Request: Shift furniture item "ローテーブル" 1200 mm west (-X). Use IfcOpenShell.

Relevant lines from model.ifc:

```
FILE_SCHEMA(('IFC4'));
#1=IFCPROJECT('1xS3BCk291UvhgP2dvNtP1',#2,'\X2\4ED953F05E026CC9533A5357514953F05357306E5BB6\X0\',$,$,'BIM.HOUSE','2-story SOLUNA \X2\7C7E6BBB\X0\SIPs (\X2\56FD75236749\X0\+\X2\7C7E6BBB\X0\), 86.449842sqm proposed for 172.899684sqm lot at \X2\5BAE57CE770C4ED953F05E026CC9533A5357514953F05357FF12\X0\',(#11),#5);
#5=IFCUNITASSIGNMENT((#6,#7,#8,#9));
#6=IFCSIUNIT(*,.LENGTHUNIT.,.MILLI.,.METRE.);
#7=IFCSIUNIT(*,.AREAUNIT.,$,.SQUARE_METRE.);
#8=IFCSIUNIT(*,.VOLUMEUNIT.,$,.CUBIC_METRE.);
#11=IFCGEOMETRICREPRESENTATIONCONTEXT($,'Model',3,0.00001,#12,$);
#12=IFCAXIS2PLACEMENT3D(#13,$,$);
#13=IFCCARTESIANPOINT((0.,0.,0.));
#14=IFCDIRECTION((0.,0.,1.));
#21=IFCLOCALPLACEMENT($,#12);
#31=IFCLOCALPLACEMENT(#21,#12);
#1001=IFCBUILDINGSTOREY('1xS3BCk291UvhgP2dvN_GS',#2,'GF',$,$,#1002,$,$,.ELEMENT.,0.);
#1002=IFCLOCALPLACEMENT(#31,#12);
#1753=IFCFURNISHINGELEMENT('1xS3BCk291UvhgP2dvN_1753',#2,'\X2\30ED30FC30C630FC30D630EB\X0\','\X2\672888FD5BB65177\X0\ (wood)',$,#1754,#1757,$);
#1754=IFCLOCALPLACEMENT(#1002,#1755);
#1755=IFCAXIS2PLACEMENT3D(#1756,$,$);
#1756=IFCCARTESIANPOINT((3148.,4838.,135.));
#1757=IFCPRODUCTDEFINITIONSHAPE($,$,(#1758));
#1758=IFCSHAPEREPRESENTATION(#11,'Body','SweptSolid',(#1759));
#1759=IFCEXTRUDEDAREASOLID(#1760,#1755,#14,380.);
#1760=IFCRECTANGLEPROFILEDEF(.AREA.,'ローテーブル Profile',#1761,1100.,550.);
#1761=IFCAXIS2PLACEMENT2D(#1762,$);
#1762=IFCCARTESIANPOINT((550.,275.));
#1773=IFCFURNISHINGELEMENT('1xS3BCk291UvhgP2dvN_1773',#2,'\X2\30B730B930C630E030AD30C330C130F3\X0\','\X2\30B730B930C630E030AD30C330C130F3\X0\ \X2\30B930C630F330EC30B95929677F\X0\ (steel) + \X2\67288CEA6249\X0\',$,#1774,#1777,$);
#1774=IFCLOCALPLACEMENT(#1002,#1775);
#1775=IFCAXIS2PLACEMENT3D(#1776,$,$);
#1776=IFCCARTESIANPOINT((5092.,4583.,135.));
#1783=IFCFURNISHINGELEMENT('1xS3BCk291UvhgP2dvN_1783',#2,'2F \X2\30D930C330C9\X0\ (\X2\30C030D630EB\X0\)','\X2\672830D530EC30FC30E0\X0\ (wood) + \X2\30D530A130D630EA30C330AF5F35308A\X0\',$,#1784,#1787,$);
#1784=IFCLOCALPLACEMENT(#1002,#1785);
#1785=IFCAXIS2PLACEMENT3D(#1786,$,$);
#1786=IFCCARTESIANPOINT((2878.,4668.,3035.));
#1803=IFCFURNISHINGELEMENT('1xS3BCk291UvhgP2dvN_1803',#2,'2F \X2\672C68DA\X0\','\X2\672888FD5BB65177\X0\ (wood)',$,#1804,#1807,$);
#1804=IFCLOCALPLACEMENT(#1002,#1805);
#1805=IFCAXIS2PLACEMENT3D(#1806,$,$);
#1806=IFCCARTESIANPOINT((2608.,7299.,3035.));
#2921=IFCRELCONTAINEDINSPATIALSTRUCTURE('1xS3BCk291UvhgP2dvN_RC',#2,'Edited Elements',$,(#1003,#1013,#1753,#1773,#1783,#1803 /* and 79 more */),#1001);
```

```python
import ifcopenshell
import ifcopenshell.api.geometry
import ifcopenshell.util.placement
import ifcopenshell.util.unit

model = ifcopenshell.open("model.ifc")
unit_scale = ifcopenshell.util.unit.calculate_unit_scale(model)

item = model.by_id(1753)
matrix = ifcopenshell.util.placement.get_local_placement(item.ObjectPlacement)
matrix[0, 3] -= 1.2 / unit_scale
ifcopenshell.api.geometry.edit_object_placement(model, product=item, matrix=matrix, is_si=False)

print(ifcopenshell.util.placement.get_local_placement(item.ObjectPlacement).round(3) + 0.0)

model.write("model_updated.ifc")
```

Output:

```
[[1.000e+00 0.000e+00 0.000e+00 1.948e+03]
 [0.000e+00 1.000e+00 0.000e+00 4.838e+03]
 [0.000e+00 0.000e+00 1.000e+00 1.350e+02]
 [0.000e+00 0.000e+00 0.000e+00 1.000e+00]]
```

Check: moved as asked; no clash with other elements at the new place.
